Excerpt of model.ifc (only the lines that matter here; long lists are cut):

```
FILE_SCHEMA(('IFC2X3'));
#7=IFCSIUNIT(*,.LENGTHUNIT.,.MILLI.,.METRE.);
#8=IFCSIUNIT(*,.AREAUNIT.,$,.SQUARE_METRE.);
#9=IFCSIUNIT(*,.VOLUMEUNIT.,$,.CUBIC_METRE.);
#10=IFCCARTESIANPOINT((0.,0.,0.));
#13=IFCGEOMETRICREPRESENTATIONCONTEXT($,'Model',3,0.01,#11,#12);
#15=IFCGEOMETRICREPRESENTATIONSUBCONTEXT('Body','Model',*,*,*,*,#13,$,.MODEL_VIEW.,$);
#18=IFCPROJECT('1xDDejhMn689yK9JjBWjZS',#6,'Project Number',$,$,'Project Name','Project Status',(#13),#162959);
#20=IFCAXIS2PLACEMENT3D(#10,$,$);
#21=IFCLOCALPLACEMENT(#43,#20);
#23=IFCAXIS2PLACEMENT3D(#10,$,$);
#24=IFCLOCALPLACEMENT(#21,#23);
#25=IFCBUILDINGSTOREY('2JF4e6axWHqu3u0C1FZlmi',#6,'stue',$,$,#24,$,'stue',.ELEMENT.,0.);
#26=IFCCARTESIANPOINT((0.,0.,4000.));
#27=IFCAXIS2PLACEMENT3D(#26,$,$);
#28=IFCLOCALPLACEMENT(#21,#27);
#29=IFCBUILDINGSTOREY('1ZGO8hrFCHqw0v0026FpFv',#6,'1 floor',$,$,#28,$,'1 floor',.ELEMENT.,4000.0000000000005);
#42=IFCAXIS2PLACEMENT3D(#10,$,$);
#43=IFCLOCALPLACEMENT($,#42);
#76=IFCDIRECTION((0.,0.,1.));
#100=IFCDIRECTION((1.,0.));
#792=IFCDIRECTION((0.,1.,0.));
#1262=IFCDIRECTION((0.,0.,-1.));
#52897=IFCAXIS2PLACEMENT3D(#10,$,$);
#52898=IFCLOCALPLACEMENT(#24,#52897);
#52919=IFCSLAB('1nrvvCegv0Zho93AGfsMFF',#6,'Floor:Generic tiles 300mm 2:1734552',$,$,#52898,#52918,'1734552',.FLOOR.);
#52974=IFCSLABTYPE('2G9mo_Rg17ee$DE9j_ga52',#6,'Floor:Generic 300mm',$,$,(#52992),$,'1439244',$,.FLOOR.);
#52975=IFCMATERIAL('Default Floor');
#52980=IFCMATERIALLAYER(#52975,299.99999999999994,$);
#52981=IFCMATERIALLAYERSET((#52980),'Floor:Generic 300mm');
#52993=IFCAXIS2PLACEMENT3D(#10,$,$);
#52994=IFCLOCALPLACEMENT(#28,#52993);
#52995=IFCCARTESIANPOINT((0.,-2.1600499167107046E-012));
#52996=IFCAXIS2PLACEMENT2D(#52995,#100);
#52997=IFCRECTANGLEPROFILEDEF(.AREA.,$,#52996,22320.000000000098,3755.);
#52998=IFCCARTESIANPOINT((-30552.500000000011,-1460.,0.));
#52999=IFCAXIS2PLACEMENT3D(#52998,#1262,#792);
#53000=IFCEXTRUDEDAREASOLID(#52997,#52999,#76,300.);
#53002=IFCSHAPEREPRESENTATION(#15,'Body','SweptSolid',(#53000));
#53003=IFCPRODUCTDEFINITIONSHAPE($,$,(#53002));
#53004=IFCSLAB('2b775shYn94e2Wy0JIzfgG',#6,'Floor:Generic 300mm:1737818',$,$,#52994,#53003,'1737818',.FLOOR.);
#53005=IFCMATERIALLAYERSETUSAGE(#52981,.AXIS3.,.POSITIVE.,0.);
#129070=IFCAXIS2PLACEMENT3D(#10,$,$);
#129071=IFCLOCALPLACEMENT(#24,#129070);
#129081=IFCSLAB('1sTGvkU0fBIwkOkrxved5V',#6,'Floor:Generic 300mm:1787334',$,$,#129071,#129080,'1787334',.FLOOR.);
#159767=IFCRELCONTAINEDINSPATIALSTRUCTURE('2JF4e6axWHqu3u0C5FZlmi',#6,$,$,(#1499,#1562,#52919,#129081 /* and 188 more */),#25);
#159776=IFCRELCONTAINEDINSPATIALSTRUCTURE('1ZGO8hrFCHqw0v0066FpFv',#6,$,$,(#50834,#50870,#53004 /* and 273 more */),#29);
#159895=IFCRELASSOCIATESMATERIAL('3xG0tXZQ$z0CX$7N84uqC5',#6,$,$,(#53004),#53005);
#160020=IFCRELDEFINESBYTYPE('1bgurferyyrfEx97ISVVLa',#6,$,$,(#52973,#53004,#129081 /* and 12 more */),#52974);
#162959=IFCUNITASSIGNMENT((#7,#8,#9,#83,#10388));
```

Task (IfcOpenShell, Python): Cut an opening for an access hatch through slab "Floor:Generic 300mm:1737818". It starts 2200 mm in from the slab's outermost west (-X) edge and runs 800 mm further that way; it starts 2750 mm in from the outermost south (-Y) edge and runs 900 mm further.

```python
import numpy as np
import ifcopenshell
import ifcopenshell.api.feature
import ifcopenshell.api.geometry
import ifcopenshell.api.root
import ifcopenshell.geom
import ifcopenshell.util.placement
import ifcopenshell.util.representation
import ifcopenshell.util.shape
import ifcopenshell.util.unit

model = ifcopenshell.open("model.ifc")
unit_scale = ifcopenshell.util.unit.calculate_unit_scale(model)
settings = ifcopenshell.geom.settings()


def volume(element):
    """Net volume in cubic metres, openings subtracted."""
    shape = ifcopenshell.geom.create_shape(settings, element)
    return ifcopenshell.util.shape.get_volume(shape.geometry)


slab = model.by_guid("2b775shYn94e2Wy0JIzfgG")
before = volume(slab)

# Extent in the slab's own axes, in metres. The edges named are its -X and -Y sides.
slab_shape = ifcopenshell.geom.create_shape(settings, slab)
vertices = ifcopenshell.util.shape.get_vertices(slab_shape.geometry)
x_min, y_min, bottom = vertices.min(axis=0)
top = vertices[:, 2].max()

opening = ifcopenshell.api.root.create_entity(model, ifc_class="IfcOpeningElement", name="Access hatch opening")
context = ifcopenshell.util.representation.get_context(model, "Model", "Body", "MODEL_VIEW")
width, depth = 0.8, 0.9
outline = [(0.0, 0.0), (width, 0.0), (width, depth), (0.0, depth), (0.0, 0.0)]
# Overshoot both faces by 50 mm so the cut is clean.
shape = ifcopenshell.api.geometry.add_slab_representation(
    model, context=context, depth=top - bottom + 0.1, polyline=outline
)
ifcopenshell.api.geometry.assign_representation(model, product=opening, representation=shape)

matrix = ifcopenshell.util.placement.get_local_placement(slab.ObjectPlacement)
matrix[:, 3] = matrix @ np.append(np.array([x_min + 2.2, y_min + 2.75, bottom - 0.05]) / unit_scale, 1.0)
ifcopenshell.api.geometry.edit_object_placement(model, product=opening, matrix=matrix, is_si=False)
ifcopenshell.api.feature.add_feature(model, feature=opening, element=slab)

after = volume(slab)

print(f"slab volume {before:.3f} -> {after:.3f} m3")

model.write("model_edited.ifc")
```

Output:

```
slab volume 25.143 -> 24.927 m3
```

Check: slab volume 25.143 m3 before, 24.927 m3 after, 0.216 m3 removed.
